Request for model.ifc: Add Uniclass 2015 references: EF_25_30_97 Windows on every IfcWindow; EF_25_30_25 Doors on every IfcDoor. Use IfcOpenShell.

First a look at what the model holds.

```python
import ifcopenshell

model = ifcopenshell.open("model.ifc")
print(model.schema)
print("classifications:", [c.Name for c in model.by_type("IfcClassification")])
for ifc_class in ("IfcDoor", "IfcRoof", "IfcStair", "IfcWall", "IfcWindow"):
    print(ifc_class, len(model.by_type(ifc_class)))
```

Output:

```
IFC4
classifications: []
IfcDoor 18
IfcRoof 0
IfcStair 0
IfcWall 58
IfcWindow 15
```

```python
import ifcopenshell
import ifcopenshell.api.classification

model = ifcopenshell.open("model.ifc")

system = ifcopenshell.api.classification.add_classification(model, classification="Uniclass 2015")

codes = {
    "IfcWindow": ("EF_25_30_97", "Windows"),
    "IfcDoor": ("EF_25_30_25", "Doors"),
}
for ifc_class, (code, name) in codes.items():
    products = model.by_type(ifc_class)
    ifcopenshell.api.classification.add_reference(
        model, products=products, classification=system, identification=code, name=name
    )
    print(code, len(products))

model.write("model_updated.ifc")
```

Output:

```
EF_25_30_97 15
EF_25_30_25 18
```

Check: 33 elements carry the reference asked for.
